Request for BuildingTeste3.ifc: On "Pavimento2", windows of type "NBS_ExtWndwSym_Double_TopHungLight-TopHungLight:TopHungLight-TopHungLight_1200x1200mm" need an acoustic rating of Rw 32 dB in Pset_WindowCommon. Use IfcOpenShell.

First a look at what the model holds.

```python
import ifcopenshell
import ifcopenshell.util.element

model = ifcopenshell.open("BuildingTeste3.ifc")
print(model.schema)
storey = next(s for s in model.by_type("IfcBuildingStorey") if s.Name == "Pavimento2")
windows = [e for e in ifcopenshell.util.element.get_decomposition(storey) if e.is_a("IfcWindow")]
seen = {}
for e in windows:
    element_type = ifcopenshell.util.element.get_type(e)
    key = (element_type.Name if element_type != e and element_type else None, ifcopenshell.util.element.get_pset(e, "Pset_WindowCommon", "AcousticRating"))
    seen[key] = seen.get(key, 0) + 1
for (name, value), count in sorted(seen.items(), key=str):
    print(count, "x", name, "|", value)
```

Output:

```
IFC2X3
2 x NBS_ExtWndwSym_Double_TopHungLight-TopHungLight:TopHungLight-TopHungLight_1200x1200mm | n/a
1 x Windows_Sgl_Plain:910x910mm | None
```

```python
import ifcopenshell
import ifcopenshell.api.pset
import ifcopenshell.util.element

model = ifcopenshell.open("BuildingTeste3.ifc")

storey = next(s for s in model.by_type("IfcBuildingStorey") if s.Name == "Pavimento2")
windows = [e for e in ifcopenshell.util.element.get_decomposition(storey) if e.is_a("IfcWindow")]

count = 0
for e in windows:
    element_type = ifcopenshell.util.element.get_type(e)
    if element_type in (None, e) or element_type.Name != "NBS_ExtWndwSym_Double_TopHungLight-TopHungLight:TopHungLight-TopHungLight_1200x1200mm":
        continue
    # add_pset returns the element's existing set when there is one.
    pset = ifcopenshell.api.pset.add_pset(model, product=e, name="Pset_WindowCommon")
    ifcopenshell.api.pset.edit_pset(model, pset=pset, properties={"AcousticRating": "Rw 32 dB"})
    count += 1

print(count, "windows updated")

model.write("BuildingTeste3-out.ifc")
```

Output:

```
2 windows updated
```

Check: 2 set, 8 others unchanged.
